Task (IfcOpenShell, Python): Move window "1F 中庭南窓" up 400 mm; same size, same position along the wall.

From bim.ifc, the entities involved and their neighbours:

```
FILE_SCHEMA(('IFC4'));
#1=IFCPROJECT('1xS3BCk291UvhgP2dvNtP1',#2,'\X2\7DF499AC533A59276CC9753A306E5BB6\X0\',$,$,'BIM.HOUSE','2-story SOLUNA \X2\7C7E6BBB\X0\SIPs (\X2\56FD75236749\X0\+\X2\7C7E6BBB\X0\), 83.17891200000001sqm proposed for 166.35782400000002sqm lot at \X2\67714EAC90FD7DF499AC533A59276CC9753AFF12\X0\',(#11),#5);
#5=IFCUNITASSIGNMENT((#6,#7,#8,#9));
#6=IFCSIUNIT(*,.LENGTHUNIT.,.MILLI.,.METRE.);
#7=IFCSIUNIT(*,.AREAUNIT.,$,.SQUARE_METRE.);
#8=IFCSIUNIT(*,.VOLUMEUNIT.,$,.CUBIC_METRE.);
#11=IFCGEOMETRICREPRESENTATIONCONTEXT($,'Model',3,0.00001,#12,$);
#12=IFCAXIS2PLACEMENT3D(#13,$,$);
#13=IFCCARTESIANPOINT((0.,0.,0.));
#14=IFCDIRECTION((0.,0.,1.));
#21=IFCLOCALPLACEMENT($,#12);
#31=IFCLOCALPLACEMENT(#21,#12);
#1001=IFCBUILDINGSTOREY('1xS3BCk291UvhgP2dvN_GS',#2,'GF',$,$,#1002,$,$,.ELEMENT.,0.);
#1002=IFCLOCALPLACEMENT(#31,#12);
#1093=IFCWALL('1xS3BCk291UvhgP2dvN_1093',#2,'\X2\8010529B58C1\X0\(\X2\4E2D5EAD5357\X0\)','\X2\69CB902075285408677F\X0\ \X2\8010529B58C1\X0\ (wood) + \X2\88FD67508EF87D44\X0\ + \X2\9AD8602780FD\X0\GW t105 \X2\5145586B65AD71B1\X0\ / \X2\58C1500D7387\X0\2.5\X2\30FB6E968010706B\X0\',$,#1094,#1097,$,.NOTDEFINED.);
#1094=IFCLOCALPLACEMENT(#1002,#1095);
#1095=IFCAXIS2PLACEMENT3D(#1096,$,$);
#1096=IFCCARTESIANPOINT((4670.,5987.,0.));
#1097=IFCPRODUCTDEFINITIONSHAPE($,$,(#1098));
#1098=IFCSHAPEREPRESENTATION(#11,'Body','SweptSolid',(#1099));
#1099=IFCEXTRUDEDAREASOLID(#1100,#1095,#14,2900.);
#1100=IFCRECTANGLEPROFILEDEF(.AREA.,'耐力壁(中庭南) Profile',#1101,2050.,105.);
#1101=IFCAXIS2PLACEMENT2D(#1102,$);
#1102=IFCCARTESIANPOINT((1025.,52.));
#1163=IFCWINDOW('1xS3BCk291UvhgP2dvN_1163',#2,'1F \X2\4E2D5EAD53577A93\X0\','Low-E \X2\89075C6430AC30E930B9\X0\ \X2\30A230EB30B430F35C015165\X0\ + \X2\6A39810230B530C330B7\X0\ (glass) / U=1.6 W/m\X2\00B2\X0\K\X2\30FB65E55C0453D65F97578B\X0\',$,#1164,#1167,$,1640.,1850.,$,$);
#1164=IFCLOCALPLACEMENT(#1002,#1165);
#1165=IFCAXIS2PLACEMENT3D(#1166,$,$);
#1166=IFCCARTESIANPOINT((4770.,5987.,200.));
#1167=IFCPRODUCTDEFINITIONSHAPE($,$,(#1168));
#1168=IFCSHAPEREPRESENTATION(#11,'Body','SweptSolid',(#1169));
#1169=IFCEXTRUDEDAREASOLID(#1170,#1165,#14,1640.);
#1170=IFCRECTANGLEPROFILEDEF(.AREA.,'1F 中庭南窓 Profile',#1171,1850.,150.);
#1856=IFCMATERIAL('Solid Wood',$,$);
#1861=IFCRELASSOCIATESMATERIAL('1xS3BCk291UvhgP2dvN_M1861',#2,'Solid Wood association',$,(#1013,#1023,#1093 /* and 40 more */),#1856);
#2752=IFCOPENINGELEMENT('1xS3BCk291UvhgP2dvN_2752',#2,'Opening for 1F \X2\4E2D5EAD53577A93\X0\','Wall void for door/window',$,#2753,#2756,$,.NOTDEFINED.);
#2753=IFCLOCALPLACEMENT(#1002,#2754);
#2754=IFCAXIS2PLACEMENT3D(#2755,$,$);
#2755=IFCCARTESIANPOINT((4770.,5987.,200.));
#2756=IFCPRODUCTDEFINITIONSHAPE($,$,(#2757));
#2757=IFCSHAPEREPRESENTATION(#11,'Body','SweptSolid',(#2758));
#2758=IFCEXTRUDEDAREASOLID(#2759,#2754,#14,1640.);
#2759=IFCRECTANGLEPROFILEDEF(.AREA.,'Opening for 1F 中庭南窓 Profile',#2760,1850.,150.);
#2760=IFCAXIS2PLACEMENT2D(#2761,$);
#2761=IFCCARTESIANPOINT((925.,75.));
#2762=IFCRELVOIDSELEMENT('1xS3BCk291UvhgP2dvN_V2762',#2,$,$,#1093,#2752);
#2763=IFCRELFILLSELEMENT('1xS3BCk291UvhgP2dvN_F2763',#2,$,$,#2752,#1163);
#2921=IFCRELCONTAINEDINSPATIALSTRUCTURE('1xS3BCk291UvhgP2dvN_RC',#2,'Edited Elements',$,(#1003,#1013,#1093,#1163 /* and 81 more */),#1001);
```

```python
import numpy as np
import ifcopenshell
import ifcopenshell.api.geometry
import ifcopenshell.util.placement
import ifcopenshell.util.unit

model = ifcopenshell.open("bim.ifc")
unit_scale = ifcopenshell.util.unit.calculate_unit_scale(model)

window = model.by_guid("1xS3BCk291UvhgP2dvN_1163")
opening = window.FillsVoids[0].RelatingOpeningElement
dz = 0.4 / unit_scale

shift = np.array([0.0, 0.0, dz])
# The window is not placed relative to its opening, so move both.
for product in (opening, window):
    matrix = ifcopenshell.util.placement.get_local_placement(product.ObjectPlacement)
    matrix[:3, 3] += shift
    ifcopenshell.api.geometry.edit_object_placement(model, product=product, matrix=matrix, is_si=False)

print(f"moved by {dz * unit_scale:+.3f} m")

model.write("bim_updated.ifc")
```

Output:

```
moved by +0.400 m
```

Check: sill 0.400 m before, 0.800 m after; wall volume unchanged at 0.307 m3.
